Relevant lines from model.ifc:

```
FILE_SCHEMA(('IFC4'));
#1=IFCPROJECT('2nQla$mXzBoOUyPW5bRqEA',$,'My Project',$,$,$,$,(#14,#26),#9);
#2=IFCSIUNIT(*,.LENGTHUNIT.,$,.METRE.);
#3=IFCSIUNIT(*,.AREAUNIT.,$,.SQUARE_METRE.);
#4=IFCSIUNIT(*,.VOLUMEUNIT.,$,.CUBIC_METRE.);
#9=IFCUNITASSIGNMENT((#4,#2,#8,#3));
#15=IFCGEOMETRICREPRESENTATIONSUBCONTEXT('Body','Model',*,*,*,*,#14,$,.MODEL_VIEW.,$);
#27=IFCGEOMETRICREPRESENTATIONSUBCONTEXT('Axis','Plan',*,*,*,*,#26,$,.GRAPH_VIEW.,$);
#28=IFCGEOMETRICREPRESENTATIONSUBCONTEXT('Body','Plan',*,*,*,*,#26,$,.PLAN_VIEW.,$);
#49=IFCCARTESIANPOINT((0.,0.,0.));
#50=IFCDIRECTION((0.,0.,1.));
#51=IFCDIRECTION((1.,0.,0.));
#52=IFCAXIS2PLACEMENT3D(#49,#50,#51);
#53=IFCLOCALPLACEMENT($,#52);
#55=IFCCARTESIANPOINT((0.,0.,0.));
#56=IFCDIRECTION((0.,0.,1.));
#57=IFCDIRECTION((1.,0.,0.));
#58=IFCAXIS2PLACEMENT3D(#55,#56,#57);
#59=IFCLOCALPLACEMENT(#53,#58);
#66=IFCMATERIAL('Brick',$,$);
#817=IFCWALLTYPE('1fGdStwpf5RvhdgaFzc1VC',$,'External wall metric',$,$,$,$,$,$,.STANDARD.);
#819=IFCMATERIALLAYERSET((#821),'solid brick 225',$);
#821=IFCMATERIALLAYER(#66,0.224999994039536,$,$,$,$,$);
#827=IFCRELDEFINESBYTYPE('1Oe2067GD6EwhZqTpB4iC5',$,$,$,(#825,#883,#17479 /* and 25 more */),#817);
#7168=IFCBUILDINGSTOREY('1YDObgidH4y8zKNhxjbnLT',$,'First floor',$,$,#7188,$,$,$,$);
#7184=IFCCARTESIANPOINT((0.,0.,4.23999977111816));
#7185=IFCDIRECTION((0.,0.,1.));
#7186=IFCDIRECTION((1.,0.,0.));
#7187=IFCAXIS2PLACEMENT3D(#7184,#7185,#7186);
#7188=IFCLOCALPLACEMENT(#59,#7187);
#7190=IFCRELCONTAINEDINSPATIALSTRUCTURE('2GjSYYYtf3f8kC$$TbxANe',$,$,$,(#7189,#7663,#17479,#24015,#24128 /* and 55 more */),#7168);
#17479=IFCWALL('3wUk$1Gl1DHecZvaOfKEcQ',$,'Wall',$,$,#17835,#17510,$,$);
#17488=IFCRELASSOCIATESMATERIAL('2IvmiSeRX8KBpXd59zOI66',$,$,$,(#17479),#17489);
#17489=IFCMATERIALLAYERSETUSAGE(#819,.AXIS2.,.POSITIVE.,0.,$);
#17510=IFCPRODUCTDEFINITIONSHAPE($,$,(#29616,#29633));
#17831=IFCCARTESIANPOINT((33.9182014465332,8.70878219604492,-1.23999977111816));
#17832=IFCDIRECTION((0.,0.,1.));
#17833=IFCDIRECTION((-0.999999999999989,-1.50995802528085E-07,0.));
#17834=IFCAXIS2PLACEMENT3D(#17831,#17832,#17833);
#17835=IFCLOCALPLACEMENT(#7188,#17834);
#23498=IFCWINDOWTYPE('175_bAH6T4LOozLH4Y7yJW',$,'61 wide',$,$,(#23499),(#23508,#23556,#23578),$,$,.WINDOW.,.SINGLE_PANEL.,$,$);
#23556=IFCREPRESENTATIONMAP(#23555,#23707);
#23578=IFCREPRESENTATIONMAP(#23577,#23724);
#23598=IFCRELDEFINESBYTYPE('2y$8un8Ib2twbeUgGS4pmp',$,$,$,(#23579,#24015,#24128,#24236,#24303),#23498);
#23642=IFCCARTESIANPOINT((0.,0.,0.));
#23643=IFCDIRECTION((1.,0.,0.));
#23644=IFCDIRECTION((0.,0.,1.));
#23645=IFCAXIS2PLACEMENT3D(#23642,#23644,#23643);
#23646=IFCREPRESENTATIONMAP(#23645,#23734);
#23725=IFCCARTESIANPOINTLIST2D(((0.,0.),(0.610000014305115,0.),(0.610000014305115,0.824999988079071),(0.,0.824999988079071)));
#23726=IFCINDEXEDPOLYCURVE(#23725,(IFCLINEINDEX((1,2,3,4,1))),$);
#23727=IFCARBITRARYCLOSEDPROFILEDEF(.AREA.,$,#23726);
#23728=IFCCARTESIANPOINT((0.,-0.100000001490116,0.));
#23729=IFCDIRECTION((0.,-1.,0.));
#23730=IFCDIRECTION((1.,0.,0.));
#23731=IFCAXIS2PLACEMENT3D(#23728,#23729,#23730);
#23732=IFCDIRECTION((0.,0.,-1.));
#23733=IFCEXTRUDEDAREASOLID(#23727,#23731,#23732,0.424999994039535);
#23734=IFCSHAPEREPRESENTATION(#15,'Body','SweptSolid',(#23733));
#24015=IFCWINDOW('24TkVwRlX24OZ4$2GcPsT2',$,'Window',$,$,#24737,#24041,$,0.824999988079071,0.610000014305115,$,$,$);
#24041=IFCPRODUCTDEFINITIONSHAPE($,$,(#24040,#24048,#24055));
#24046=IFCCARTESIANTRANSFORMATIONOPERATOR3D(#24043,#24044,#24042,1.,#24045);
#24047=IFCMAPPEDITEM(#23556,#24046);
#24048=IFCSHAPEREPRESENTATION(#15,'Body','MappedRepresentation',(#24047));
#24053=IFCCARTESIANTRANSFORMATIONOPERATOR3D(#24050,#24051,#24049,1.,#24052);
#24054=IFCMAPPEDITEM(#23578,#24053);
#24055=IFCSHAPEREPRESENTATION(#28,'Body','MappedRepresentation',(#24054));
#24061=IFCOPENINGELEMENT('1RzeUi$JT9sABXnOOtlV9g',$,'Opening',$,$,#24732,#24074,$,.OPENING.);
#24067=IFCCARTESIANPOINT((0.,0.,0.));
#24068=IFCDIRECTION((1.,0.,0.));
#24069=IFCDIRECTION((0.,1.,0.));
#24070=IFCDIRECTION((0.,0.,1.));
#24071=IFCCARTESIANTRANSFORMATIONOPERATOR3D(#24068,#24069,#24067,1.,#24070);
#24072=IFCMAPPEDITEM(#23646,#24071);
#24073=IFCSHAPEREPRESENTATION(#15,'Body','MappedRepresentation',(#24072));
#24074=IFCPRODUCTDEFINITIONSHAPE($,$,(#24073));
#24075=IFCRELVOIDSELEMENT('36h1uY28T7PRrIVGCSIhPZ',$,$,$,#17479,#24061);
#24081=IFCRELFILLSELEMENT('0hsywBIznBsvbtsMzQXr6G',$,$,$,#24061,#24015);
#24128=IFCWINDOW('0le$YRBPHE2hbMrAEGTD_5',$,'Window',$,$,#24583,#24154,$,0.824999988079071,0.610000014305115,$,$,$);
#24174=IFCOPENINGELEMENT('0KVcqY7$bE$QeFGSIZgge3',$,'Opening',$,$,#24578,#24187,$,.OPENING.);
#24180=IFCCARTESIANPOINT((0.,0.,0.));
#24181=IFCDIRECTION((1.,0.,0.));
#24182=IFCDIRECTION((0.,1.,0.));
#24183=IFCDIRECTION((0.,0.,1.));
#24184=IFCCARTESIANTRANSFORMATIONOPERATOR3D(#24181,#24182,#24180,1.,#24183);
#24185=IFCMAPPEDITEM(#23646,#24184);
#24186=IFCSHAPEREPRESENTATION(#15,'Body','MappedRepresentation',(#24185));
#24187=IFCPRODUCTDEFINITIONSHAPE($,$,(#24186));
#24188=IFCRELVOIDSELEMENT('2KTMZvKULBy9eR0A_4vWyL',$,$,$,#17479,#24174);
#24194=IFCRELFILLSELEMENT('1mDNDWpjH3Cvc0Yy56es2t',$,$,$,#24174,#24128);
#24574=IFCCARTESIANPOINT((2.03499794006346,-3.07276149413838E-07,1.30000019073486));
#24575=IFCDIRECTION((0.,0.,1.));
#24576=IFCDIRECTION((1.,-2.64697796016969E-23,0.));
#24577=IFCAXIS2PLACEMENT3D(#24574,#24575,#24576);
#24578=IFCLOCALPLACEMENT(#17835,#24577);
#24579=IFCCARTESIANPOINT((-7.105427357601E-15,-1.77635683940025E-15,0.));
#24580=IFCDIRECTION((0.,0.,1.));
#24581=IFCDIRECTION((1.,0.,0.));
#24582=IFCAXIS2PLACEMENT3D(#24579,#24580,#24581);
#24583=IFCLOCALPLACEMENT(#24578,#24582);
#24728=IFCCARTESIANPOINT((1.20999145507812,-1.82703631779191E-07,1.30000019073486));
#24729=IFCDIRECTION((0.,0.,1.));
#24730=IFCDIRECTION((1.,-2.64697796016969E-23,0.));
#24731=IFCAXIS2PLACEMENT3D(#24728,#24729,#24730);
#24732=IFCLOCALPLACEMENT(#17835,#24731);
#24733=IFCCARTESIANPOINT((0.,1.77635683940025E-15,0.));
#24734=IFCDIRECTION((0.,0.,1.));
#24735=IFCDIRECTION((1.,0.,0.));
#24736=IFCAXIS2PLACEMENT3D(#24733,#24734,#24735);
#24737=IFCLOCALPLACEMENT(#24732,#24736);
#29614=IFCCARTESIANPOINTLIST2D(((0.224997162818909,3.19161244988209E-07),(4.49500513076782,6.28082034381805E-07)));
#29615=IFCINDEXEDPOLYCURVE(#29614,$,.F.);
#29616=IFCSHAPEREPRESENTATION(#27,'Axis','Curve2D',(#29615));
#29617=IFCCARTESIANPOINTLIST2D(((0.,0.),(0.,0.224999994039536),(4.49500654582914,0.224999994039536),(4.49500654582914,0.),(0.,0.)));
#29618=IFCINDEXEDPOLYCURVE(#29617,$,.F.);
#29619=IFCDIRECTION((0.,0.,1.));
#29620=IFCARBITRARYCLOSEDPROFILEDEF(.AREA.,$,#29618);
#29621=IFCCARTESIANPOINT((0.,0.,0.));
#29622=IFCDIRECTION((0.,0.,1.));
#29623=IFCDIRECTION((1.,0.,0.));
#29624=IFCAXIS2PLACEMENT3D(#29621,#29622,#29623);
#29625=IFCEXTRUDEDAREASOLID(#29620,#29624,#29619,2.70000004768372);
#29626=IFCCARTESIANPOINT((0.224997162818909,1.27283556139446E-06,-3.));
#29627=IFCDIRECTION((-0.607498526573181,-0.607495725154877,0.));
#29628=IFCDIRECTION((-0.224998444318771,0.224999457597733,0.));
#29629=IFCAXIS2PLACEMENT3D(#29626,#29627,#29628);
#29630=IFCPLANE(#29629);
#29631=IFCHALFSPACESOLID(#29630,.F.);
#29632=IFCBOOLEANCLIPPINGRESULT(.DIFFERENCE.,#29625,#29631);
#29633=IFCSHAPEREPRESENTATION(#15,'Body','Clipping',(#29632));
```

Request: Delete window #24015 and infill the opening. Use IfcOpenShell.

```python
import ifcopenshell
import ifcopenshell.api.feature
import ifcopenshell.api.root
import ifcopenshell.geom
import ifcopenshell.util.shape

model = ifcopenshell.open("model.ifc")
settings = ifcopenshell.geom.settings()


def volume(element):
    """Net volume in cubic metres, openings subtracted."""
    shape = ifcopenshell.geom.create_shape(settings, element)
    return ifcopenshell.util.shape.get_volume(shape.geometry)


window = model.by_id(24015)
opening = window.FillsVoids[0].RelatingOpeningElement
wall = opening.VoidsElements[0].RelatingBuildingElement
before = volume(wall)

ifcopenshell.api.root.remove_product(model, product=window)
ifcopenshell.api.feature.remove_feature(model, feature=opening)

after = volume(wall)

print(f"wall volume {before:.3f} -> {after:.3f} m3")

model.write("model-out.ifc")
```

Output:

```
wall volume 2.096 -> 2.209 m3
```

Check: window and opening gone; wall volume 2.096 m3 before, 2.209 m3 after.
